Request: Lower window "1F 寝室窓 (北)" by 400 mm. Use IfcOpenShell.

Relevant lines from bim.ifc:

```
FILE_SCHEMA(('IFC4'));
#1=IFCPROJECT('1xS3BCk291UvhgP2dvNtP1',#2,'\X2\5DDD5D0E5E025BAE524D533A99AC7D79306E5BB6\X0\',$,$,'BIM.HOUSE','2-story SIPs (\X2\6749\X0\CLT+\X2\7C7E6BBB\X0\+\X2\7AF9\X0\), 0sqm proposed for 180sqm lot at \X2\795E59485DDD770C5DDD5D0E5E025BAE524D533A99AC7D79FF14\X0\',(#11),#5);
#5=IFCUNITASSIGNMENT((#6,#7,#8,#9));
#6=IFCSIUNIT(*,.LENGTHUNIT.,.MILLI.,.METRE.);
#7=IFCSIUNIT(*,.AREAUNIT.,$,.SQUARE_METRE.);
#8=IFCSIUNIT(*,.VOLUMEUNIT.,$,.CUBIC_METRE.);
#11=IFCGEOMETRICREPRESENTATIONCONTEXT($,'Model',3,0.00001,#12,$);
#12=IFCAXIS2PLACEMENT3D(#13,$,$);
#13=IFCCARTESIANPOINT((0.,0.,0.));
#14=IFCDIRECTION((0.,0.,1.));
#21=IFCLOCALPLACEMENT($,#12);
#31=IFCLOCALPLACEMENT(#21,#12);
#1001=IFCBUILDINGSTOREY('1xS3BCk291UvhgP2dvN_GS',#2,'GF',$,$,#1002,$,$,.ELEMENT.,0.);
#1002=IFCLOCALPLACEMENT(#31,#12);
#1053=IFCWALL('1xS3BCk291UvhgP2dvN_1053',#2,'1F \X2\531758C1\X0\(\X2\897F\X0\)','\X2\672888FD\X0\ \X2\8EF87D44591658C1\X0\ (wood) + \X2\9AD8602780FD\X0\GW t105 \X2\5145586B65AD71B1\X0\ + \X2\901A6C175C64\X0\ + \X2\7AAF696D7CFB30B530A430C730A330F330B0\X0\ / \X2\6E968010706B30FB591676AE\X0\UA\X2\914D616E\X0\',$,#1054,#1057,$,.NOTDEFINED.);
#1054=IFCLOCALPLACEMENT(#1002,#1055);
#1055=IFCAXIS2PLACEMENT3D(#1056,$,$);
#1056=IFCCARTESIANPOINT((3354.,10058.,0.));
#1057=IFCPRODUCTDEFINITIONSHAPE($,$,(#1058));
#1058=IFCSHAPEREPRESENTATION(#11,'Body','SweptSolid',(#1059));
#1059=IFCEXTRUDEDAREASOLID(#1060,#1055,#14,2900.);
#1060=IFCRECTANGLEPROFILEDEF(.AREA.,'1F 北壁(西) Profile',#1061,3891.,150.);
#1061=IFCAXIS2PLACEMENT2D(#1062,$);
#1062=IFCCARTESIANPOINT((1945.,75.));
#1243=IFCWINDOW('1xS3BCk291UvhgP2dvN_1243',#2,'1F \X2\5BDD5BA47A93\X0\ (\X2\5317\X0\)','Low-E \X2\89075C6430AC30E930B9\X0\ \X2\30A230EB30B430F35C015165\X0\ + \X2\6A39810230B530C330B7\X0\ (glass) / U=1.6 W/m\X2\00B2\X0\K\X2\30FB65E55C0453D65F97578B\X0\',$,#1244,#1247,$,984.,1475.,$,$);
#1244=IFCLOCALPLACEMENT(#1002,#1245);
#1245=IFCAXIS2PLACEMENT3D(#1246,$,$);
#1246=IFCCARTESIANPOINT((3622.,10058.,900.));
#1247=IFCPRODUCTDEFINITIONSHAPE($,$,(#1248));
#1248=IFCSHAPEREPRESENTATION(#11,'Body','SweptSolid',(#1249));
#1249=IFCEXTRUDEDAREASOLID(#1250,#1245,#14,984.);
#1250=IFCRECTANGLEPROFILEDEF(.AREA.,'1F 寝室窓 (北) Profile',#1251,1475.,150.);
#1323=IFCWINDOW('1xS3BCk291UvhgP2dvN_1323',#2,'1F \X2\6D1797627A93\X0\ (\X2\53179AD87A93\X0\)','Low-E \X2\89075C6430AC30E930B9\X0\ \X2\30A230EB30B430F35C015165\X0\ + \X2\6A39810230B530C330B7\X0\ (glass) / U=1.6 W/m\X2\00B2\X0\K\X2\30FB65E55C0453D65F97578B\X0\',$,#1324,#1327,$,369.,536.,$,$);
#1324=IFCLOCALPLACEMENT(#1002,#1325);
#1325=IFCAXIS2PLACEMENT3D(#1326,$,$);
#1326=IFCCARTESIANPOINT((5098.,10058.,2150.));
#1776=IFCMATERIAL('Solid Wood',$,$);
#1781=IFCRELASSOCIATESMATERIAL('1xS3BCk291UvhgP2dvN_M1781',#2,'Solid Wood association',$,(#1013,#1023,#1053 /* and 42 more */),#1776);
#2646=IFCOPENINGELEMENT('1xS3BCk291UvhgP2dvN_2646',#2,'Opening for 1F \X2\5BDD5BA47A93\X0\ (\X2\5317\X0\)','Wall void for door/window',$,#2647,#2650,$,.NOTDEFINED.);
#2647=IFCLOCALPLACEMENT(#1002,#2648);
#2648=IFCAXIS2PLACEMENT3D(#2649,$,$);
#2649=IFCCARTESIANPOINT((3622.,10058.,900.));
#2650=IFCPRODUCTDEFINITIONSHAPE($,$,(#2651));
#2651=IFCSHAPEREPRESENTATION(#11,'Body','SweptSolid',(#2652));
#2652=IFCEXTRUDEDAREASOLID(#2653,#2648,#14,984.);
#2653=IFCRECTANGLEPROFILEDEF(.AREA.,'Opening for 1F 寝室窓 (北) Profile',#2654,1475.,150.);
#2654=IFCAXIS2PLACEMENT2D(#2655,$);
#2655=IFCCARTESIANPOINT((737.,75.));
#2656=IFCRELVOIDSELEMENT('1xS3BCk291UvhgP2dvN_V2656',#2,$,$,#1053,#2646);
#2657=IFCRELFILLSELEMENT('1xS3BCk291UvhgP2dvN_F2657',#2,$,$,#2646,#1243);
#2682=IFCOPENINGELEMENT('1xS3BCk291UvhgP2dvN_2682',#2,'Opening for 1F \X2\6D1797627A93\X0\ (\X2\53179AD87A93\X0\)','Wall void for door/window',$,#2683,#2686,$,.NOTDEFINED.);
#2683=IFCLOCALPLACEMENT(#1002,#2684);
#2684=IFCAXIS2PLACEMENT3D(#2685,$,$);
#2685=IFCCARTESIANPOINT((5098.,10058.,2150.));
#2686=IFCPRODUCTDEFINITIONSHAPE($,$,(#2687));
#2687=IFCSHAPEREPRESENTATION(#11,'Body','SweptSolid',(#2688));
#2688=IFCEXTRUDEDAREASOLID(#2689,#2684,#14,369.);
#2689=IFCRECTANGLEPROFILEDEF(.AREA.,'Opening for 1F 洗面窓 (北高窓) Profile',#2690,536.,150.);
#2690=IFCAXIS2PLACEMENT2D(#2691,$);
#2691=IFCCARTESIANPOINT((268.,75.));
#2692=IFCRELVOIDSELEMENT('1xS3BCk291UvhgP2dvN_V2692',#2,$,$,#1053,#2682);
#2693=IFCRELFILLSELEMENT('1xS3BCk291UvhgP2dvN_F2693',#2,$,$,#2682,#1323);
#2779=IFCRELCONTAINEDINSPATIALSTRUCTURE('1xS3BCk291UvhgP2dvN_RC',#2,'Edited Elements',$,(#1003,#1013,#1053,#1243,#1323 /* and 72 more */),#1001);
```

```python
import numpy as np
import ifcopenshell
import ifcopenshell.api.geometry
import ifcopenshell.util.placement
import ifcopenshell.util.unit

model = ifcopenshell.open("bim.ifc")
unit_scale = ifcopenshell.util.unit.calculate_unit_scale(model)

window = model.by_guid("1xS3BCk291UvhgP2dvN_1243")
opening = window.FillsVoids[0].RelatingOpeningElement
dz = -400.0

shift = np.array([0.0, 0.0, dz])
# The window is not placed relative to its opening, so move both.
for product in (opening, window):
    matrix = ifcopenshell.util.placement.get_local_placement(product.ObjectPlacement)
    matrix[:3, 3] += shift
    ifcopenshell.api.geometry.edit_object_placement(model, product=product, matrix=matrix, is_si=False)

print(f"moved by {dz * unit_scale:+.3f} m")

model.write("bim_v2.ifc")
```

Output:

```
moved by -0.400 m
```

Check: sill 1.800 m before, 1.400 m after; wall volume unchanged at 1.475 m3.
